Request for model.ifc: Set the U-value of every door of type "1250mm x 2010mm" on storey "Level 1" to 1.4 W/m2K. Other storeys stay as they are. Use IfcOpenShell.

First a look at what the model holds.

```python
import ifcopenshell
import ifcopenshell.util.element

model = ifcopenshell.open("model.ifc")
print(model.schema)
storey = next(s for s in model.by_type("IfcBuildingStorey") if s.Name == "Level 1")
doors = [e for e in ifcopenshell.util.element.get_decomposition(storey) if e.is_a("IfcDoor")]
seen = {}
for e in doors:
    element_type = ifcopenshell.util.element.get_type(e)
    key = (element_type.Name if element_type != e and element_type else None, ifcopenshell.util.element.get_pset(e, "Pset_DoorCommon", "ThermalTransmittance"))
    seen[key] = seen.get(key, 0) + 1
for (name, value), count in sorted(seen.items(), key=str):
    print(count, "x", name, "|", value)
```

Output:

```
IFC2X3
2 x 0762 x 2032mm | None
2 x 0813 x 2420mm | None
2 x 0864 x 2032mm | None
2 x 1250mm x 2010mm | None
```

```python
import ifcopenshell
import ifcopenshell.api.pset
import ifcopenshell.util.element

model = ifcopenshell.open("model.ifc")

storey = next(s for s in model.by_type("IfcBuildingStorey") if s.Name == "Level 1")
doors = [e for e in ifcopenshell.util.element.get_decomposition(storey) if e.is_a("IfcDoor")]

count = 0
for e in doors:
    element_type = ifcopenshell.util.element.get_type(e)
    if element_type in (None, e) or element_type.Name != "1250mm x 2010mm":
        continue
    # add_pset returns the element's existing set when there is one.
    pset = ifcopenshell.api.pset.add_pset(model, product=e, name="Pset_DoorCommon")
    ifcopenshell.api.pset.edit_pset(model, pset=pset, properties={"ThermalTransmittance": 1.4})
    count += 1

print(count, "doors updated")

model.write("model_rev.ifc")
```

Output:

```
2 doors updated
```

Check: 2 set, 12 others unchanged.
